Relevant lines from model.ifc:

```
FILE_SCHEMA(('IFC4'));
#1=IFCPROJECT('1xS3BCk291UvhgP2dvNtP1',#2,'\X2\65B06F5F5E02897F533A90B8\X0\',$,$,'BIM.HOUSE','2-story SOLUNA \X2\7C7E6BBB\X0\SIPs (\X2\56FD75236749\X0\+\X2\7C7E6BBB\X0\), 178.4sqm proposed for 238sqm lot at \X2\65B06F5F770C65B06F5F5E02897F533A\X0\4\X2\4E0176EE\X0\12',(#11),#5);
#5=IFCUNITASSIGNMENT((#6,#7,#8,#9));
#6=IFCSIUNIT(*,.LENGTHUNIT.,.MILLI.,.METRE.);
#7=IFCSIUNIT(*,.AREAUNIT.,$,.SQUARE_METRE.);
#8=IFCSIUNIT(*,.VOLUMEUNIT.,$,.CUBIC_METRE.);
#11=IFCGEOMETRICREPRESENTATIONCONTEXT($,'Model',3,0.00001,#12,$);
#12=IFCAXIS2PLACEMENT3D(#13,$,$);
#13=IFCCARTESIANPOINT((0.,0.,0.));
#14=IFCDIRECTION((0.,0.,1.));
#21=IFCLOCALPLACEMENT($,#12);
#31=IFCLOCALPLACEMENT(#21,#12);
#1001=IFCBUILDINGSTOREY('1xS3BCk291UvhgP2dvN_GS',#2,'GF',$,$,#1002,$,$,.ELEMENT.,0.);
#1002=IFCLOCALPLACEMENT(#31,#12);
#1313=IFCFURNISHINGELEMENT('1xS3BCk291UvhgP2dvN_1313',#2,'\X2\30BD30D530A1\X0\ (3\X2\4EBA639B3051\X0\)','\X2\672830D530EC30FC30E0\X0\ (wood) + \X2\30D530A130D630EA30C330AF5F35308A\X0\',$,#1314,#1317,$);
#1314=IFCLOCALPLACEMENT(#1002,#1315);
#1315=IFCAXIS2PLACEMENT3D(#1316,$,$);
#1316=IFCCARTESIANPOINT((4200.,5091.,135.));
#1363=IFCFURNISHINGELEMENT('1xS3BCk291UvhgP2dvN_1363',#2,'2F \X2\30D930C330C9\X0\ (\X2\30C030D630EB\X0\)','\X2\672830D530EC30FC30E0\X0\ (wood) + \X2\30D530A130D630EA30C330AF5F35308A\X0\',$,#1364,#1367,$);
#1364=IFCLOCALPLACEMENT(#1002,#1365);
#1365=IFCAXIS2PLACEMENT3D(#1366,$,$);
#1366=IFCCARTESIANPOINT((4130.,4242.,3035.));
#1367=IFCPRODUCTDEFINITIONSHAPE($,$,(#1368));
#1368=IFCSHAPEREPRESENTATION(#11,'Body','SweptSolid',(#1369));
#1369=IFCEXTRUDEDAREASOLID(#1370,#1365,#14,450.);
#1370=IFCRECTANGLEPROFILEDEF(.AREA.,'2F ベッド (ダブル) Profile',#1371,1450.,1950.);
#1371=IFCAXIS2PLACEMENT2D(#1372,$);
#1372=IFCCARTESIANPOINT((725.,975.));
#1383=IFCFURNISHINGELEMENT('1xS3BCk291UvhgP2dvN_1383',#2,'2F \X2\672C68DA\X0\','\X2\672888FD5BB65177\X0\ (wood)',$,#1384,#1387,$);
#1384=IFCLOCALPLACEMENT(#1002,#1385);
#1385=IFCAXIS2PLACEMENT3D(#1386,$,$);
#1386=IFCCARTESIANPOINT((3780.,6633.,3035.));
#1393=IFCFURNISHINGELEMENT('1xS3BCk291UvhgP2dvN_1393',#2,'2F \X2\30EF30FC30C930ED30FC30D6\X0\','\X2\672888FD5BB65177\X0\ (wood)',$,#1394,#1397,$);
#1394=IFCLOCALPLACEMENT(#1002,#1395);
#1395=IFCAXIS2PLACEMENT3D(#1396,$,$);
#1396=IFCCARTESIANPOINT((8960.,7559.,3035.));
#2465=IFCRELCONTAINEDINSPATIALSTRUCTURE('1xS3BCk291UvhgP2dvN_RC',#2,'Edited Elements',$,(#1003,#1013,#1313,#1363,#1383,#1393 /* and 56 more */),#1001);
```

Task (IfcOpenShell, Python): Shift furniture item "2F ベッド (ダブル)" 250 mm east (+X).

```python
import ifcopenshell
import ifcopenshell.api.geometry
import ifcopenshell.util.placement
import ifcopenshell.util.unit

model = ifcopenshell.open("model.ifc")
unit_scale = ifcopenshell.util.unit.calculate_unit_scale(model)

item = model.by_id(1363)
matrix = ifcopenshell.util.placement.get_local_placement(item.ObjectPlacement)
matrix[0, 3] += 0.25 / unit_scale
ifcopenshell.api.geometry.edit_object_placement(model, product=item, matrix=matrix, is_si=False)

print(ifcopenshell.util.placement.get_local_placement(item.ObjectPlacement).round(3) + 0.0)

model.write("model-out.ifc")
```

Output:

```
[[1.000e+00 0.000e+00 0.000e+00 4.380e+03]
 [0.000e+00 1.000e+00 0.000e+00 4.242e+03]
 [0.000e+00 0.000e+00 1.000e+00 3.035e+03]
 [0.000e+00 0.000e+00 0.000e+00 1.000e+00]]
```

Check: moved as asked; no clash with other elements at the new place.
